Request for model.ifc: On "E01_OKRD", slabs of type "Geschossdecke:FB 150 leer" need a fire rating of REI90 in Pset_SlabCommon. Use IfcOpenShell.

First a look at what the model holds.

```python
import ifcopenshell
import ifcopenshell.util.element

model = ifcopenshell.open("model.ifc")
print(model.schema)
storey = next(s for s in model.by_type("IfcBuildingStorey") if s.Name == "E01_OKRD")
slabs = [e for e in ifcopenshell.util.element.get_decomposition(storey) if e.is_a("IfcSlab")]
seen = {}
for e in slabs:
    element_type = ifcopenshell.util.element.get_type(e)
    key = (element_type.Name if element_type != e and element_type else None, ifcopenshell.util.element.get_pset(e, "Pset_SlabCommon", "FireRating"))
    seen[key] = seen.get(key, 0) + 1
for (name, value), count in sorted(seen.items(), key=str):
    print(count, "x", name, "|", value)
```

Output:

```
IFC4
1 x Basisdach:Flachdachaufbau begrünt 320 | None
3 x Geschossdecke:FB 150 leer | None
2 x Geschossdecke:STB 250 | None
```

```python
import ifcopenshell
import ifcopenshell.api.pset
import ifcopenshell.util.element

model = ifcopenshell.open("model.ifc")

storey = next(s for s in model.by_type("IfcBuildingStorey") if s.Name == "E01_OKRD")
slabs = [e for e in ifcopenshell.util.element.get_decomposition(storey) if e.is_a("IfcSlab")]

count = 0
for e in slabs:
    element_type = ifcopenshell.util.element.get_type(e)
    if element_type in (None, e) or element_type.Name != "Geschossdecke:FB 150 leer":
        continue
    # add_pset returns the element's existing set when there is one.
    pset = ifcopenshell.api.pset.add_pset(model, product=e, name="Pset_SlabCommon")
    ifcopenshell.api.pset.edit_pset(model, pset=pset, properties={"FireRating": "REI90"})
    count += 1

print(count, "slabs updated")

model.write("model_edited.ifc")
```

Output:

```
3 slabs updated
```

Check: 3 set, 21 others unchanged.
